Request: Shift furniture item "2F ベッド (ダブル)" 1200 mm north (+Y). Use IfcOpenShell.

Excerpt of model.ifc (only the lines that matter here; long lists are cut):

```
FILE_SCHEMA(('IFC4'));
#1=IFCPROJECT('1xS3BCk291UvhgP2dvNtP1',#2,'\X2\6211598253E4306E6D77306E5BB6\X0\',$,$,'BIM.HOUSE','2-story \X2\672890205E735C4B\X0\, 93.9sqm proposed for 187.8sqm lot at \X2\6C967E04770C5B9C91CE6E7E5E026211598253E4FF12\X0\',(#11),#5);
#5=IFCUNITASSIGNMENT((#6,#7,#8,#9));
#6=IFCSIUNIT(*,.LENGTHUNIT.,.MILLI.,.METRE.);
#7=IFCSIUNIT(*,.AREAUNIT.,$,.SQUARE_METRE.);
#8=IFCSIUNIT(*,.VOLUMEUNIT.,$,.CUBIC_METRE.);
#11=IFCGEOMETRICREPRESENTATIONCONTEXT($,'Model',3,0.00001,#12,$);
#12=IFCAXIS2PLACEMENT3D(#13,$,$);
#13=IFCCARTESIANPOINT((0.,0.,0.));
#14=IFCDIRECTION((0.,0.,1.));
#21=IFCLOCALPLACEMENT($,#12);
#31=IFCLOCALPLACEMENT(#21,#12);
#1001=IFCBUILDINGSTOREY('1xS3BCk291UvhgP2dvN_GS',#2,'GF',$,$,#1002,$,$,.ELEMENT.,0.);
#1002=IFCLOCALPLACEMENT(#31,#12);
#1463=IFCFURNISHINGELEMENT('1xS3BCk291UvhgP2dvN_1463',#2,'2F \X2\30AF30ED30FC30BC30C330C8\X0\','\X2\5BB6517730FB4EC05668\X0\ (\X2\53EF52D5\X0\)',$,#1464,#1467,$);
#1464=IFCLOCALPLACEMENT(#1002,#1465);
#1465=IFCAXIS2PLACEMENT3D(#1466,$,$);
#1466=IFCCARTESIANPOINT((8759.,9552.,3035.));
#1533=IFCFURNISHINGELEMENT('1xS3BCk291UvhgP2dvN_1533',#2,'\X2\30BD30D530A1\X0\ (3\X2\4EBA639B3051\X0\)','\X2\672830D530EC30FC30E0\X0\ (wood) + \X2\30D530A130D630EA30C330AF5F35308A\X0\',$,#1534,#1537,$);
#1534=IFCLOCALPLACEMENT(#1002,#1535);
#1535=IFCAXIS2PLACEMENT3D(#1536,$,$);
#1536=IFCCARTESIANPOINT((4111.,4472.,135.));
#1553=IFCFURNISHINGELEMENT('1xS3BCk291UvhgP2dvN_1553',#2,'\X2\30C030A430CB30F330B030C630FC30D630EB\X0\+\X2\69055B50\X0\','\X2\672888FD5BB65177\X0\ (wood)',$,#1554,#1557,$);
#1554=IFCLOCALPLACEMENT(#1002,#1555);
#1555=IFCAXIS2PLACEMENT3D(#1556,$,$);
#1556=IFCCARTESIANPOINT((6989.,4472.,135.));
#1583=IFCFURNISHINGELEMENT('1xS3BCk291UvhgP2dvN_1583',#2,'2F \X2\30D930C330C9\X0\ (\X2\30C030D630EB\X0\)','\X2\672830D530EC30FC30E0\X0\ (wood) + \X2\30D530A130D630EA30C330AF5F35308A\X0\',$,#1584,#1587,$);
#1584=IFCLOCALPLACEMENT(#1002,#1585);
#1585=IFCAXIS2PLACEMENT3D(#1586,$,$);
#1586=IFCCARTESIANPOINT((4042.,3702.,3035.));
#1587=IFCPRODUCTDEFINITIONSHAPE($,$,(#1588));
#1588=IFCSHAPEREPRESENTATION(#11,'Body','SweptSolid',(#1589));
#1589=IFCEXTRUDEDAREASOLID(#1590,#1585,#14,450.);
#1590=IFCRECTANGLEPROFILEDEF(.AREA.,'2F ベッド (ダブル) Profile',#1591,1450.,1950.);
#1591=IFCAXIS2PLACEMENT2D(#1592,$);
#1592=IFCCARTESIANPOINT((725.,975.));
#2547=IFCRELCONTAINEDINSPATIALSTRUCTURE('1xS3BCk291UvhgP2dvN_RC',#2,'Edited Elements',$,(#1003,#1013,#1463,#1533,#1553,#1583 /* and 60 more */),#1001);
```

```python
import ifcopenshell
import ifcopenshell.api.geometry
import ifcopenshell.util.placement
import ifcopenshell.util.unit

model = ifcopenshell.open("model.ifc")
unit_scale = ifcopenshell.util.unit.calculate_unit_scale(model)

item = model.by_guid("1xS3BCk291UvhgP2dvN_1583")
matrix = ifcopenshell.util.placement.get_local_placement(item.ObjectPlacement)
matrix[1, 3] += 1.2 / unit_scale
ifcopenshell.api.geometry.edit_object_placement(model, product=item, matrix=matrix, is_si=False)

print(ifcopenshell.util.placement.get_local_placement(item.ObjectPlacement).round(3) + 0.0)

model.write("model_updated.ifc")
```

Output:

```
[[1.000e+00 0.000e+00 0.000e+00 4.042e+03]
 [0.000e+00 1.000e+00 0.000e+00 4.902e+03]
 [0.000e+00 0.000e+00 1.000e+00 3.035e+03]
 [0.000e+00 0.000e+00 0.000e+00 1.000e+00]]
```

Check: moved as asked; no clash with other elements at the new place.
